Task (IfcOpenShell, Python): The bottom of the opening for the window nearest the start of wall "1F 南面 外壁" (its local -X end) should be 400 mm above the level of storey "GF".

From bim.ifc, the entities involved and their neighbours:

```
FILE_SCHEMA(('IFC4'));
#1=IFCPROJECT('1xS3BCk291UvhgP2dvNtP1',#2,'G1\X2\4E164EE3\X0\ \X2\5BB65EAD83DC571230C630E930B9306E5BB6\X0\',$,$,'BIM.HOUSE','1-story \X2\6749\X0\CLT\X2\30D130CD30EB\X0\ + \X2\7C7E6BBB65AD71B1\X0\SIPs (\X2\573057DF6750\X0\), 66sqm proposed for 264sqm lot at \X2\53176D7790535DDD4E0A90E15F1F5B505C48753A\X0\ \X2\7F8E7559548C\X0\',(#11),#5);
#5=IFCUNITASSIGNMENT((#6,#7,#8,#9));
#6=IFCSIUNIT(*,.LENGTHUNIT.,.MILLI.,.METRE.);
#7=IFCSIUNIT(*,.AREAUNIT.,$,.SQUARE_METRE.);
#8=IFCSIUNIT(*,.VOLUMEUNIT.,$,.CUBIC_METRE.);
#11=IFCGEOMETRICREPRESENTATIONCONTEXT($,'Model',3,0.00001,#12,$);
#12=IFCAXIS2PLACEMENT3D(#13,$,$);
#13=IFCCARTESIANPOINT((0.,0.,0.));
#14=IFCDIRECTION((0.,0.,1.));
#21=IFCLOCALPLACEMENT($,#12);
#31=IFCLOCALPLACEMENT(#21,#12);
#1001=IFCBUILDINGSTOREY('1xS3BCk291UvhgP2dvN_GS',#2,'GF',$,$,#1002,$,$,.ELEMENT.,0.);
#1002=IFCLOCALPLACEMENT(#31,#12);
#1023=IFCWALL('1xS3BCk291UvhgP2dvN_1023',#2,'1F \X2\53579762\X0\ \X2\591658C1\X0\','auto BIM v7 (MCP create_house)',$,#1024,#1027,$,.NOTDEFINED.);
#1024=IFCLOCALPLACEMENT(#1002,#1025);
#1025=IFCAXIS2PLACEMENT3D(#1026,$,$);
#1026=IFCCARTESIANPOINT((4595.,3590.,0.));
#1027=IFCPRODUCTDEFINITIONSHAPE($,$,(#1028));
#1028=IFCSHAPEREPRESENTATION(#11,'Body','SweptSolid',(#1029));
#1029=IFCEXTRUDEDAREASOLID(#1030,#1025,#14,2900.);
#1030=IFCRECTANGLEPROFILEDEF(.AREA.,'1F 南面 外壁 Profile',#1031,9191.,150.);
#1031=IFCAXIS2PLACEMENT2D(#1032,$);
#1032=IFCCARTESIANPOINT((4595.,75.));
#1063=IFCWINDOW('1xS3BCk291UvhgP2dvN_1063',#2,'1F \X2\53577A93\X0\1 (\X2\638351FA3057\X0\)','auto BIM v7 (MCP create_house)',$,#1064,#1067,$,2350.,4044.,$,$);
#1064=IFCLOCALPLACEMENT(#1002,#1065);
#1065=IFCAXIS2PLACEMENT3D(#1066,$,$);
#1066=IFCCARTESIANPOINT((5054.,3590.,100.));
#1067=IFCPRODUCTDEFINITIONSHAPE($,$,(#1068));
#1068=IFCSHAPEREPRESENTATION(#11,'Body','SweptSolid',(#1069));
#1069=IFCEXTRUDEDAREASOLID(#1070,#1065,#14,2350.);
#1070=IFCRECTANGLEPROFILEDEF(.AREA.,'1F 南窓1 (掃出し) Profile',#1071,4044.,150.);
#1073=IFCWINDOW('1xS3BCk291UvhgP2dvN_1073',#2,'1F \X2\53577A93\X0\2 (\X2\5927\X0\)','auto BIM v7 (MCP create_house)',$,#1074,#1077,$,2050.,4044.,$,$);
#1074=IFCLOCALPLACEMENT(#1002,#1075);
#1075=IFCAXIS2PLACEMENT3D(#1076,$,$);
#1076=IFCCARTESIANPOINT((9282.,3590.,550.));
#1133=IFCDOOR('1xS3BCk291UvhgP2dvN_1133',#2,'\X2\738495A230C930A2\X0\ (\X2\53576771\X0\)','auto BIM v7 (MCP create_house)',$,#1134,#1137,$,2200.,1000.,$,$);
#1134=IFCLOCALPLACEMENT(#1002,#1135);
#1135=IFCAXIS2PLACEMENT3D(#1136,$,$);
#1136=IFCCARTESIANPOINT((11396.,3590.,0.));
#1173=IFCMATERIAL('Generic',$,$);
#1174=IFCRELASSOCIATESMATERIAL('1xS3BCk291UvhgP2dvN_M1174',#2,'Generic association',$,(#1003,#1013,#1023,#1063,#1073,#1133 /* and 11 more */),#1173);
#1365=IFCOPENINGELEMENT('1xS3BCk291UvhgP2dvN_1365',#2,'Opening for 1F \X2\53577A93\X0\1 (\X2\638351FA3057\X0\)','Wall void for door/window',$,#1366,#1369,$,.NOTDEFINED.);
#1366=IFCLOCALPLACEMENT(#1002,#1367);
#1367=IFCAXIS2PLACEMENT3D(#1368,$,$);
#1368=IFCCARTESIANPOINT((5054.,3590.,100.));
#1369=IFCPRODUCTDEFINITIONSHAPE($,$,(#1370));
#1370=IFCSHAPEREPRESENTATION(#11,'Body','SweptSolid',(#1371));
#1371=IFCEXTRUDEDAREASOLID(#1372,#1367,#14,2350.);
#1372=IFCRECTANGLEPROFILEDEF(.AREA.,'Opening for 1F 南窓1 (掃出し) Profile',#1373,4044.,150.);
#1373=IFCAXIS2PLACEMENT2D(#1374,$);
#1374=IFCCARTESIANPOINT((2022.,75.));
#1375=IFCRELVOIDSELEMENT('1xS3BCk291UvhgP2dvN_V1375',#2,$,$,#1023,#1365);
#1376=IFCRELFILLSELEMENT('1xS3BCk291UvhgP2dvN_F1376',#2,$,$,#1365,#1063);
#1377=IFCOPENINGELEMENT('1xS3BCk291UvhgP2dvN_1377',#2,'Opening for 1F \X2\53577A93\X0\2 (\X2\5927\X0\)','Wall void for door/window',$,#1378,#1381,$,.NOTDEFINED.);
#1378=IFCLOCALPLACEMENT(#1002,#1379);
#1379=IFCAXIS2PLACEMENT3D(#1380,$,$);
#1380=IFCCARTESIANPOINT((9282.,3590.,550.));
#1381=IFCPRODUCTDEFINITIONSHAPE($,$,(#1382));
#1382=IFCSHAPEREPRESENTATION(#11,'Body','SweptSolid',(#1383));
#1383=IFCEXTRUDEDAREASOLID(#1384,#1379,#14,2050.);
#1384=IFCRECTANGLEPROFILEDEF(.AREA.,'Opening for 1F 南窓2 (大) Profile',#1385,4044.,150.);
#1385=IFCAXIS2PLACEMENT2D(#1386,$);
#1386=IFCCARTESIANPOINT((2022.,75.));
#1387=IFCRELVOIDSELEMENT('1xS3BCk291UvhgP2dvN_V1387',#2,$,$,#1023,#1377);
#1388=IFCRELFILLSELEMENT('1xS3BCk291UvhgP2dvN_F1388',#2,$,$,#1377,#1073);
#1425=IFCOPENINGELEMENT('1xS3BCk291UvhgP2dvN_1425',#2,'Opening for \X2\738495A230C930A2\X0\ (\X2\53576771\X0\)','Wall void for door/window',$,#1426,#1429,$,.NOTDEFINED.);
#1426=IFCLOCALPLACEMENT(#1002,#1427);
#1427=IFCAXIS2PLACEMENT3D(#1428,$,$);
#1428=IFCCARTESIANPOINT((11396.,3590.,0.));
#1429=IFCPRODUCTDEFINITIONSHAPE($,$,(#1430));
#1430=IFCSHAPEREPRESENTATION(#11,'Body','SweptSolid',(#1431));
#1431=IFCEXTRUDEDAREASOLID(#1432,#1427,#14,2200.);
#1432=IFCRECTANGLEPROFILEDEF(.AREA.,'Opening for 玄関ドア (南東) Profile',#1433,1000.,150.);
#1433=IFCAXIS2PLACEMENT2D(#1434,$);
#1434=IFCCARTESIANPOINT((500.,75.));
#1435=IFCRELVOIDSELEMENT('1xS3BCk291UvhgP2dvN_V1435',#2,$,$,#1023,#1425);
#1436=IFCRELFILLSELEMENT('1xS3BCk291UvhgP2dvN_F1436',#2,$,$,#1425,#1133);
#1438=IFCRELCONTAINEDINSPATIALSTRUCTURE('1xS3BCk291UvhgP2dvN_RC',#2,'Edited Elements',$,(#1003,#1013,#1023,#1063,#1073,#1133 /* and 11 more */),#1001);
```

```python
import numpy as np
import ifcopenshell
import ifcopenshell.api.geometry
import ifcopenshell.geom
import ifcopenshell.util.element
import ifcopenshell.util.placement
import ifcopenshell.util.shape
import ifcopenshell.util.unit

model = ifcopenshell.open("bim.ifc")
unit_scale = ifcopenshell.util.unit.calculate_unit_scale(model)

window = model.by_guid("1xS3BCk291UvhgP2dvN_1063")
opening = window.FillsVoids[0].RelatingOpeningElement
storey = ifcopenshell.util.element.get_container(window, ifc_class="IfcBuildingStorey")
level = ifcopenshell.util.placement.get_local_placement(storey.ObjectPlacement)[2, 3]

# The opening's origin need not be at the sill, so measure its lowest point.
shape = ifcopenshell.geom.create_shape(ifcopenshell.geom.settings(), opening)
bottom = ifcopenshell.util.shape.get_shape_bottom_elevation(shape, shape.geometry) / unit_scale
dz = level + 0.4 / unit_scale - bottom

shift = np.array([0.0, 0.0, dz])
# The window is not placed relative to its opening, so move both.
for product in (opening, window):
    matrix = ifcopenshell.util.placement.get_local_placement(product.ObjectPlacement)
    matrix[:3, 3] += shift
    ifcopenshell.api.geometry.edit_object_placement(model, product=product, matrix=matrix, is_si=False)

print(f"moved by {dz * unit_scale:+.3f} m")

model.write("bim-out.ifc")
```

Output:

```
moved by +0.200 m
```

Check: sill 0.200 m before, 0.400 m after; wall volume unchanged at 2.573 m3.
